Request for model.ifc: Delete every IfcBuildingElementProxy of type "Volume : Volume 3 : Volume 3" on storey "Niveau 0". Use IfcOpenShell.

First a look at what the model holds.

```python
import ifcopenshell
import ifcopenshell.util.element

model = ifcopenshell.open("model.ifc")
print(model.schema)
storey = next(s for s in model.by_type("IfcBuildingStorey") if s.Name == "Niveau 0")
proxies = [e for e in ifcopenshell.util.element.get_decomposition(storey) if e.is_a("IfcBuildingElementProxy")]
seen = {}
for e in proxies:
    element_type = ifcopenshell.util.element.get_type(e)
    name = element_type.Name if element_type not in (None, e) else None
    seen[name] = seen.get(name, 0) + 1
for name, count in sorted(seen.items(), key=str):
    print(count, "x", name)
```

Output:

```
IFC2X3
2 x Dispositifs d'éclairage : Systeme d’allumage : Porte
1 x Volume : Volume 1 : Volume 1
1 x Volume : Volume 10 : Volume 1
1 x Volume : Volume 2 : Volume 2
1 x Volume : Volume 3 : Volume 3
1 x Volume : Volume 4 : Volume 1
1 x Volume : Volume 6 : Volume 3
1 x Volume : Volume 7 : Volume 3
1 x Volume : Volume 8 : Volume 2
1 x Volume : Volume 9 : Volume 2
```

```python
import ifcopenshell
import ifcopenshell.api.root
import ifcopenshell.util.element

model = ifcopenshell.open("model.ifc")

storey = next(s for s in model.by_type("IfcBuildingStorey") if s.Name == "Niveau 0")
proxies = [e for e in ifcopenshell.util.element.get_decomposition(storey) if e.is_a("IfcBuildingElementProxy")]
targets = [e for e in proxies if (t := ifcopenshell.util.element.get_type(e)) not in (None, e) and t.Name == "Volume : Volume 3 : Volume 3"]

for e in targets:
    ifcopenshell.api.root.remove_product(model, product=e)
print(len(targets), "removed")

model.write("model-out.ifc")
```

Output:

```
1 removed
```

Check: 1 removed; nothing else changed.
